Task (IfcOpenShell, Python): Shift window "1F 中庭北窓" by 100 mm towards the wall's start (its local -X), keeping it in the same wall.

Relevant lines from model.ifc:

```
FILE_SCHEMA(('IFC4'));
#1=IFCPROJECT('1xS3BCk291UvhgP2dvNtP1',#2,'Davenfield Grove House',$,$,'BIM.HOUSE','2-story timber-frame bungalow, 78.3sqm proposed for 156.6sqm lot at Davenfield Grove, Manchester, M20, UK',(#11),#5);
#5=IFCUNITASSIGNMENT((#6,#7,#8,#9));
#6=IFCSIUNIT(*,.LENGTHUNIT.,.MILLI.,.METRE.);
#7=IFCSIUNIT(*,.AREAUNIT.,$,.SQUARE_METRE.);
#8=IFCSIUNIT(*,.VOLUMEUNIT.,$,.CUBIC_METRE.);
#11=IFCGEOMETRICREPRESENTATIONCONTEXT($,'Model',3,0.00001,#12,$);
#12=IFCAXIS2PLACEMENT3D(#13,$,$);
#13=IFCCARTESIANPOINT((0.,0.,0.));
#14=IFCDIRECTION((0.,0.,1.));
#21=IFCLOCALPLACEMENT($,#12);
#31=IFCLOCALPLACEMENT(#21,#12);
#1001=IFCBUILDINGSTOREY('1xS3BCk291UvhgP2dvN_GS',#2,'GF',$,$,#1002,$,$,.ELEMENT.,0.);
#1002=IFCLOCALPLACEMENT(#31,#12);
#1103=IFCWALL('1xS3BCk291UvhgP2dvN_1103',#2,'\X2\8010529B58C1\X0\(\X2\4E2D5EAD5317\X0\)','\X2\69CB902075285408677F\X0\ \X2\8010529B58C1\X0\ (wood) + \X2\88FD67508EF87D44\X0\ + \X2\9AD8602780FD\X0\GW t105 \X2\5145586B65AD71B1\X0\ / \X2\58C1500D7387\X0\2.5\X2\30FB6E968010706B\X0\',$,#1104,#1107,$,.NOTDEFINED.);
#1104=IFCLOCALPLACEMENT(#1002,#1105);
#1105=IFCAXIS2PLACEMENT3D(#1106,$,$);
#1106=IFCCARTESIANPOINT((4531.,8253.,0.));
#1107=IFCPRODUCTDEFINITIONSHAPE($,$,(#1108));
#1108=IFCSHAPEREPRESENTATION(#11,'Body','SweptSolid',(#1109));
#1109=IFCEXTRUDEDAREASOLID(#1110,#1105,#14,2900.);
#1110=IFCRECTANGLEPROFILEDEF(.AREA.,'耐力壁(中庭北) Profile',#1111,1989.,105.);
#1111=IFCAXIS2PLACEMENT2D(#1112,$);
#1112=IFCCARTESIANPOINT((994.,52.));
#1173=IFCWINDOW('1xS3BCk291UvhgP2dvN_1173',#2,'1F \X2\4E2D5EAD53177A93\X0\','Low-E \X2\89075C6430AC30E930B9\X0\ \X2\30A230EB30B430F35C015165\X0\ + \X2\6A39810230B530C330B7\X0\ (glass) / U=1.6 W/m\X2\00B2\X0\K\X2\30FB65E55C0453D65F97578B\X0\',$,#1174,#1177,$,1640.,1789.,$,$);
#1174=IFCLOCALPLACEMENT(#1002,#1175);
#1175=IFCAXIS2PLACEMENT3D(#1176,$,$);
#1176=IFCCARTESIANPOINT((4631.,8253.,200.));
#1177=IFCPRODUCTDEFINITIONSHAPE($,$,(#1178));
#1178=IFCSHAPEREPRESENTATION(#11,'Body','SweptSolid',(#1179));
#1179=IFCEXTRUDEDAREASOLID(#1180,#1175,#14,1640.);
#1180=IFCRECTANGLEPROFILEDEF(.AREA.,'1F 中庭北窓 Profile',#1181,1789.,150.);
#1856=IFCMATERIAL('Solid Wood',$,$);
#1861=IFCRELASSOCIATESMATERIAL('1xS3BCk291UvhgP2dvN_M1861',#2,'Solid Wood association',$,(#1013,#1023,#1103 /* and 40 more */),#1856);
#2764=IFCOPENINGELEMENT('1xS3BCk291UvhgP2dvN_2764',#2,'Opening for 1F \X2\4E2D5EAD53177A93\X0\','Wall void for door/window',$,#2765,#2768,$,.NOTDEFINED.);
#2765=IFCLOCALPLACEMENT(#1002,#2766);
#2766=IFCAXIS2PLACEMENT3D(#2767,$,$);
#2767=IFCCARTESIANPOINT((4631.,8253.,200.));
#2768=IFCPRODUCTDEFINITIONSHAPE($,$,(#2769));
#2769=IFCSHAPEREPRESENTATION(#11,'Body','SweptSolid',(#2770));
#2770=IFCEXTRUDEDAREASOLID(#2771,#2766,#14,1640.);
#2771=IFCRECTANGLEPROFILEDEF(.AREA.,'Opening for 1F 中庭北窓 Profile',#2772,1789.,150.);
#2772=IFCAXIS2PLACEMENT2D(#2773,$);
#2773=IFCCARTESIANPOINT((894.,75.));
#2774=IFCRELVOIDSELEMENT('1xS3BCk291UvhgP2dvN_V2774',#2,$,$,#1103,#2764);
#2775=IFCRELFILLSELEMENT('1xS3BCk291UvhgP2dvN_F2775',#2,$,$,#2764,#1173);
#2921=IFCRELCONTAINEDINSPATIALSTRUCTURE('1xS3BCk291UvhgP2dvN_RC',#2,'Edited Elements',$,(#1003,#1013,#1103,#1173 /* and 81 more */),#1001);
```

```python
import ifcopenshell
import ifcopenshell.api.geometry
import ifcopenshell.util.placement

model = ifcopenshell.open("model.ifc")

window = model.by_guid("1xS3BCk291UvhgP2dvN_1173")
opening = window.FillsVoids[0].RelatingOpeningElement
wall = opening.VoidsElements[0].RelatingBuildingElement

wall_matrix = ifcopenshell.util.placement.get_local_placement(wall.ObjectPlacement)
shift = wall_matrix[:3, 0] * -100.0
before = ifcopenshell.util.placement.get_local_placement(window.ObjectPlacement)[:3, 3].copy()

# The window is not placed relative to its opening, so move both.
for product in (opening, window):
    matrix = ifcopenshell.util.placement.get_local_placement(product.ObjectPlacement)
    matrix[:3, 3] += shift
    ifcopenshell.api.geometry.edit_object_placement(model, product=product, matrix=matrix, is_si=False)

after = ifcopenshell.util.placement.get_local_placement(window.ObjectPlacement)[:3, 3]
print("window moved by", (after - before).round(3) + 0.0)

model.write("model-out.ifc")
```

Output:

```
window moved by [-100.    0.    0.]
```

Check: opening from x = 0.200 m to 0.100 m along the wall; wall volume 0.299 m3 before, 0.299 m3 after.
